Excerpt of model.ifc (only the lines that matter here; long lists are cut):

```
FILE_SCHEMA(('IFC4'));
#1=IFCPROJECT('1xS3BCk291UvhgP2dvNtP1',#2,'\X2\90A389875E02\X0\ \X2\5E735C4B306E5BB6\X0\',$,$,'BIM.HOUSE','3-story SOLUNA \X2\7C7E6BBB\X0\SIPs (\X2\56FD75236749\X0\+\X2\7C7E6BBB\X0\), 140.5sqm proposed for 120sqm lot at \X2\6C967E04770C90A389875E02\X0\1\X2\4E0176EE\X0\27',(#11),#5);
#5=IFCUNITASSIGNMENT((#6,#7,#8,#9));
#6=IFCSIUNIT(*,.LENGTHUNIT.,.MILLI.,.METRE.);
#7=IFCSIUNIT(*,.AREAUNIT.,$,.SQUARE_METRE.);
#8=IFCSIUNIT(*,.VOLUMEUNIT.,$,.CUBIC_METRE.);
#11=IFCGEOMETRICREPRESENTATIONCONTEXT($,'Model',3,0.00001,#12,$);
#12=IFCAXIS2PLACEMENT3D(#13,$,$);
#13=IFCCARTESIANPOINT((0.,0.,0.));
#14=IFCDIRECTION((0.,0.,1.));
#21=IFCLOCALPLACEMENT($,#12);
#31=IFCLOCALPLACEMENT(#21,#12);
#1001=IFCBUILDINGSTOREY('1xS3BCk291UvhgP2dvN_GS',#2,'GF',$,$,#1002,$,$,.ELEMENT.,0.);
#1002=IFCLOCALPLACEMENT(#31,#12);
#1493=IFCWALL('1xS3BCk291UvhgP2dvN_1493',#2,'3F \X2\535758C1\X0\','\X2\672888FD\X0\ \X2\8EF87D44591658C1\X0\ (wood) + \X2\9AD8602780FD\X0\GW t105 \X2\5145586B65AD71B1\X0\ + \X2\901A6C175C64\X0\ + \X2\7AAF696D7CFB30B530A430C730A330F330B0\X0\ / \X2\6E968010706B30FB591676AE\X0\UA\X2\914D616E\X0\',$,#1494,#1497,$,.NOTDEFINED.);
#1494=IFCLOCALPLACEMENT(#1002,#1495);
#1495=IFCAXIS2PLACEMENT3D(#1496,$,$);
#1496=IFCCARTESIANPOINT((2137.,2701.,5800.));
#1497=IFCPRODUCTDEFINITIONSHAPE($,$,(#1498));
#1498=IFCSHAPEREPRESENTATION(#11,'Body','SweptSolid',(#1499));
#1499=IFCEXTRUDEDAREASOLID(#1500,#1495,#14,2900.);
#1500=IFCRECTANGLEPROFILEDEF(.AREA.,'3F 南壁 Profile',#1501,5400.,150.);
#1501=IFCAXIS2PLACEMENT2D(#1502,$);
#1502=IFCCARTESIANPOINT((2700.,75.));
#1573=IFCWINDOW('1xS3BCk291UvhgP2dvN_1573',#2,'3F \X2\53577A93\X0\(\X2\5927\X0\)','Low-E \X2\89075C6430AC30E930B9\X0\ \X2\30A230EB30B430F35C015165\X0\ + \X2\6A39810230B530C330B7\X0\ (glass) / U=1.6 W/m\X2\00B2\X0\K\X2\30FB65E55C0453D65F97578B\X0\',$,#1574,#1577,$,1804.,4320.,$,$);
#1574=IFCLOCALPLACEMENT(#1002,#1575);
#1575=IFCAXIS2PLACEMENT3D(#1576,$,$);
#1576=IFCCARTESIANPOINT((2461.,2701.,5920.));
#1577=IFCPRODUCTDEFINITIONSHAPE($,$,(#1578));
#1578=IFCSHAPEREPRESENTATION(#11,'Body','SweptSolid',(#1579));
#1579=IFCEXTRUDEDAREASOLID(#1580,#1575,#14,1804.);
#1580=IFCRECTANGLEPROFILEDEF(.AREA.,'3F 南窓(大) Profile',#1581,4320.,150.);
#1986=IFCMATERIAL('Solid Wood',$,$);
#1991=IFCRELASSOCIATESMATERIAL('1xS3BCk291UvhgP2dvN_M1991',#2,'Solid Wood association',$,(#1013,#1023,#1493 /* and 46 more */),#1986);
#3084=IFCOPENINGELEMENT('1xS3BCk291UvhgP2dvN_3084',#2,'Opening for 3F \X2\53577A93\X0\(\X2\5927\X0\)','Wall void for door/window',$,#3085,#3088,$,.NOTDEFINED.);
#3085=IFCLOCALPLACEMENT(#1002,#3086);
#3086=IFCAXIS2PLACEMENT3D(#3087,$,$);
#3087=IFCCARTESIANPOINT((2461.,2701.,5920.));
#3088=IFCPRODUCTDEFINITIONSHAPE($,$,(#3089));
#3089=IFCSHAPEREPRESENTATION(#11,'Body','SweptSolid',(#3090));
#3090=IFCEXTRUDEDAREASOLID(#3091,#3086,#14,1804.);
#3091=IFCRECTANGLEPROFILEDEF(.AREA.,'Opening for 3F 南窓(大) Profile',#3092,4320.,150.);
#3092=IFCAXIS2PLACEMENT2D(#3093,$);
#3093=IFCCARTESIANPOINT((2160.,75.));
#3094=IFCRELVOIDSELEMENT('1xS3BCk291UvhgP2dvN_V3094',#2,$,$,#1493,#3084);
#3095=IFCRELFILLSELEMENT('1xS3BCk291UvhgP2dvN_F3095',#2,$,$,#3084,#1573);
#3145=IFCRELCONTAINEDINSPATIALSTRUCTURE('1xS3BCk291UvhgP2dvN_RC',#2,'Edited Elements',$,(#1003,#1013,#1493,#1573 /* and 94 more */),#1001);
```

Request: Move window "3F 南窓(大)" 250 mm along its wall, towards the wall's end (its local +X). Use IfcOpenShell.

```python
import ifcopenshell
import ifcopenshell.api.geometry
import ifcopenshell.util.placement

model = ifcopenshell.open("model.ifc")

window = model.by_guid("1xS3BCk291UvhgP2dvN_1573")
opening = window.FillsVoids[0].RelatingOpeningElement
wall = opening.VoidsElements[0].RelatingBuildingElement

wall_matrix = ifcopenshell.util.placement.get_local_placement(wall.ObjectPlacement)
shift = wall_matrix[:3, 0] * 250.0
before = ifcopenshell.util.placement.get_local_placement(window.ObjectPlacement)[:3, 3].copy()

# The window is not placed relative to its opening, so move both.
for product in (opening, window):
    matrix = ifcopenshell.util.placement.get_local_placement(product.ObjectPlacement)
    matrix[:3, 3] += shift
    ifcopenshell.api.geometry.edit_object_placement(model, product=product, matrix=matrix, is_si=False)

after = ifcopenshell.util.placement.get_local_placement(window.ObjectPlacement)[:3, 3]
print("window moved by", (after - before).round(3) + 0.0)

model.write("model_rev.ifc")
```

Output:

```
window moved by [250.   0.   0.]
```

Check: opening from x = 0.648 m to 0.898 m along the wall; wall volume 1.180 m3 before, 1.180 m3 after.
